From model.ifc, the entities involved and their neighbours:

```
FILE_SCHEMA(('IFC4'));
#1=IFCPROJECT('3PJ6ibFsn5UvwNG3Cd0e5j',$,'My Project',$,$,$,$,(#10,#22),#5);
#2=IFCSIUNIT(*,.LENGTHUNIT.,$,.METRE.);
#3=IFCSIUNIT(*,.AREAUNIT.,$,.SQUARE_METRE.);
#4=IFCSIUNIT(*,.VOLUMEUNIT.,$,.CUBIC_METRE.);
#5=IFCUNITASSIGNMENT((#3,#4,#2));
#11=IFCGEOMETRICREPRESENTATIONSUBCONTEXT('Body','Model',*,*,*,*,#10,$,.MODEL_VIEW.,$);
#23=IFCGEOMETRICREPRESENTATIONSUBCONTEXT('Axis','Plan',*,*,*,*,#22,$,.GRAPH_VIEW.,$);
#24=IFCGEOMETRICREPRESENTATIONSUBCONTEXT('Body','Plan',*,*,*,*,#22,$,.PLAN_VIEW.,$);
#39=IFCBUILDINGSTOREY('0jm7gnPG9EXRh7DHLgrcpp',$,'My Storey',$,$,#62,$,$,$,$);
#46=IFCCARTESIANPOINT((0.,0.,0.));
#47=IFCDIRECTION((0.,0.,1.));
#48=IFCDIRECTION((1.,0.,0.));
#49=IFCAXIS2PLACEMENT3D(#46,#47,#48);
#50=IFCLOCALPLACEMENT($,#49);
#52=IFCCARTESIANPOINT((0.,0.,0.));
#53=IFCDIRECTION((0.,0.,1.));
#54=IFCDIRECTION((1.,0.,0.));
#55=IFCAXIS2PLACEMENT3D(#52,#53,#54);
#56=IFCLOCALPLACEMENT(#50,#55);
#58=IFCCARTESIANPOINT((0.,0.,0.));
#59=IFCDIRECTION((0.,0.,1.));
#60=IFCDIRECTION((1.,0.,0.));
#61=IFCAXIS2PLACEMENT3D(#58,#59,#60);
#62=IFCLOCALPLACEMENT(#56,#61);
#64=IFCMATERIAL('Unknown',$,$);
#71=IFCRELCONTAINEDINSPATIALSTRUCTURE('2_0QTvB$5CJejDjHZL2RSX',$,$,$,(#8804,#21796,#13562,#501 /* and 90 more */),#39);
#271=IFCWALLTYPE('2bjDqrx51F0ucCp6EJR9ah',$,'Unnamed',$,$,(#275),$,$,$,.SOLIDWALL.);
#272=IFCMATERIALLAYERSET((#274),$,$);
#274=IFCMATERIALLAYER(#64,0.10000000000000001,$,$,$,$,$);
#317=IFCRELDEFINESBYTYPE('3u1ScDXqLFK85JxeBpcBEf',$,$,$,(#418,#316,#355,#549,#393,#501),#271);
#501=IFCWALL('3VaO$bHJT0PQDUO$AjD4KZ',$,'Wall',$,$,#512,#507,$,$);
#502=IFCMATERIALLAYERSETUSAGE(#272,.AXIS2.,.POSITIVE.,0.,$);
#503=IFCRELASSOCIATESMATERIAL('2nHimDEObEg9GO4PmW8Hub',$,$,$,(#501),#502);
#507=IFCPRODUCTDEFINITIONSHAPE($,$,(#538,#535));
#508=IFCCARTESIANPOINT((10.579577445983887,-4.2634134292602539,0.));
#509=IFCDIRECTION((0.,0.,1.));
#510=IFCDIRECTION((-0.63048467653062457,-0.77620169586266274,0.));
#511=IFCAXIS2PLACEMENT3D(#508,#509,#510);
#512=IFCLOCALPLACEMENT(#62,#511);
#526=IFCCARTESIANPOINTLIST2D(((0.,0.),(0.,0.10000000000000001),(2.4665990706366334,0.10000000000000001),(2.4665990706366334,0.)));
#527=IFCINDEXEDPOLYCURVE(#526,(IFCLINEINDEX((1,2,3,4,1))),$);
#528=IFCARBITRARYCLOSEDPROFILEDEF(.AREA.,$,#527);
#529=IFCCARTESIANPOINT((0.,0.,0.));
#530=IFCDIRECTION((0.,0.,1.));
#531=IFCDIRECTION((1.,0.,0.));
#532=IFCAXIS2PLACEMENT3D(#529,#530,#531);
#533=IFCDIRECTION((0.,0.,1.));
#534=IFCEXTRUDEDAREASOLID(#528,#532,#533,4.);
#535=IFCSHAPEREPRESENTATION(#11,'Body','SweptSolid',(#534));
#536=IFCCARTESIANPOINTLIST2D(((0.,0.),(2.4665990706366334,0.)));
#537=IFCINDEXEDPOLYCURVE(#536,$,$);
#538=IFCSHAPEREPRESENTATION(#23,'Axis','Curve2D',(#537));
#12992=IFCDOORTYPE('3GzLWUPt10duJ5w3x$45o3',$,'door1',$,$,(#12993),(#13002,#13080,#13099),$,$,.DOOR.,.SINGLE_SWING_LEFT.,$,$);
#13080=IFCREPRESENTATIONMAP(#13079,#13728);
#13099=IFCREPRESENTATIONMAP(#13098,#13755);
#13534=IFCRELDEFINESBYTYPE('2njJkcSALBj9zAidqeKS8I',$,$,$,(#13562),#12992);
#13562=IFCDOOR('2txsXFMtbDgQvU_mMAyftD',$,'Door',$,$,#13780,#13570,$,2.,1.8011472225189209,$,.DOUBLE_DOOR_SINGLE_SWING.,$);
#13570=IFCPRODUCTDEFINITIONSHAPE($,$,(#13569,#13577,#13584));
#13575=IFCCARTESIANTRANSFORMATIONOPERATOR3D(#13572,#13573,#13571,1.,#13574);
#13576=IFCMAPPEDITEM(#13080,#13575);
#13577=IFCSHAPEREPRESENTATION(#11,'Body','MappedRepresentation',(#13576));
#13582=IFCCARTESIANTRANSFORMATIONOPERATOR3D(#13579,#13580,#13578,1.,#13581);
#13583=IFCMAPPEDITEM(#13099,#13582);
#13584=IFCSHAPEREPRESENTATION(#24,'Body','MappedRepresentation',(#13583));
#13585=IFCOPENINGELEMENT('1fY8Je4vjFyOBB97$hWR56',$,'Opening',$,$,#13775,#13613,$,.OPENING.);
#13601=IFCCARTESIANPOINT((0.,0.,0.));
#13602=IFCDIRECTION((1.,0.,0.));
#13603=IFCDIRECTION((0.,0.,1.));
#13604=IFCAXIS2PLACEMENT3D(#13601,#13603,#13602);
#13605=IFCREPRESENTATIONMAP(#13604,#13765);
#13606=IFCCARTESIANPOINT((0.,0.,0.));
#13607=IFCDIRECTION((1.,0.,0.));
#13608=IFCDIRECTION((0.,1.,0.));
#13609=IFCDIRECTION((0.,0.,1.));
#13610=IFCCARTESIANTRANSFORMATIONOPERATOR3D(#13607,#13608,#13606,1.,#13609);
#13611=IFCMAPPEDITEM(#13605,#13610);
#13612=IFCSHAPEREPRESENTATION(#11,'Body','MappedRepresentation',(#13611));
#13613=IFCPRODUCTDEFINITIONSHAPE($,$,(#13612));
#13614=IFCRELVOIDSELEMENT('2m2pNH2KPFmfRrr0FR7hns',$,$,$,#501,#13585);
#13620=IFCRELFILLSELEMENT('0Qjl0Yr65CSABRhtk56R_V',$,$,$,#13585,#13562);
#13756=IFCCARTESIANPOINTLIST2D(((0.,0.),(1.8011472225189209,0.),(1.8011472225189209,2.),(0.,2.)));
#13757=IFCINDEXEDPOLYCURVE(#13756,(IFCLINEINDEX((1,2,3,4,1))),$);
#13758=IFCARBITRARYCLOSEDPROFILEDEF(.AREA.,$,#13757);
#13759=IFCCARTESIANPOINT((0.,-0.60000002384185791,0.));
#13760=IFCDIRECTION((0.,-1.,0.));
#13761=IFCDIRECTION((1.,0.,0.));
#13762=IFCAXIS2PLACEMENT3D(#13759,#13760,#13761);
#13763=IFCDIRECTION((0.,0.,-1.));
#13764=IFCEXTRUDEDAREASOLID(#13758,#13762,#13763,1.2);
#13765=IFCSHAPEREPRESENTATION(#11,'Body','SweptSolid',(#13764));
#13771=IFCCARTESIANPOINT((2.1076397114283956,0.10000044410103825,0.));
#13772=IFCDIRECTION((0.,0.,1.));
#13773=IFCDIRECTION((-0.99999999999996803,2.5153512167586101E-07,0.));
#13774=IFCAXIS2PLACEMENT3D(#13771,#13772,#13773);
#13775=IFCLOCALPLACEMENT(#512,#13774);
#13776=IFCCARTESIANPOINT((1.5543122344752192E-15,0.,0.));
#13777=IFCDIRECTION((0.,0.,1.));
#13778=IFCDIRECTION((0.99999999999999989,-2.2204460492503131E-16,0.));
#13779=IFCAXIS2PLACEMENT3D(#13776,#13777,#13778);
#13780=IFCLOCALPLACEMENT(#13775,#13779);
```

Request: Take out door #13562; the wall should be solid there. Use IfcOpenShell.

```python
import ifcopenshell
import ifcopenshell.api.feature
import ifcopenshell.api.root
import ifcopenshell.geom
import ifcopenshell.util.shape

model = ifcopenshell.open("model.ifc")
settings = ifcopenshell.geom.settings()


def volume(element):
    """Net volume in cubic metres, openings subtracted."""
    shape = ifcopenshell.geom.create_shape(settings, element)
    return ifcopenshell.util.shape.get_volume(shape.geometry)


door = model.by_guid("2txsXFMtbDgQvU_mMAyftD")
opening = door.FillsVoids[0].RelatingOpeningElement
wall = opening.VoidsElements[0].RelatingBuildingElement
before = volume(wall)

ifcopenshell.api.root.remove_product(model, product=door)
ifcopenshell.api.feature.remove_feature(model, feature=opening)

after = volume(wall)

print(f"wall volume {before:.3f} -> {after:.3f} m3")

model.write("model_rev.ifc")
```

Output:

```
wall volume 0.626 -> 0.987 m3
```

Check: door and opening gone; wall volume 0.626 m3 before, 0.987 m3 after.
